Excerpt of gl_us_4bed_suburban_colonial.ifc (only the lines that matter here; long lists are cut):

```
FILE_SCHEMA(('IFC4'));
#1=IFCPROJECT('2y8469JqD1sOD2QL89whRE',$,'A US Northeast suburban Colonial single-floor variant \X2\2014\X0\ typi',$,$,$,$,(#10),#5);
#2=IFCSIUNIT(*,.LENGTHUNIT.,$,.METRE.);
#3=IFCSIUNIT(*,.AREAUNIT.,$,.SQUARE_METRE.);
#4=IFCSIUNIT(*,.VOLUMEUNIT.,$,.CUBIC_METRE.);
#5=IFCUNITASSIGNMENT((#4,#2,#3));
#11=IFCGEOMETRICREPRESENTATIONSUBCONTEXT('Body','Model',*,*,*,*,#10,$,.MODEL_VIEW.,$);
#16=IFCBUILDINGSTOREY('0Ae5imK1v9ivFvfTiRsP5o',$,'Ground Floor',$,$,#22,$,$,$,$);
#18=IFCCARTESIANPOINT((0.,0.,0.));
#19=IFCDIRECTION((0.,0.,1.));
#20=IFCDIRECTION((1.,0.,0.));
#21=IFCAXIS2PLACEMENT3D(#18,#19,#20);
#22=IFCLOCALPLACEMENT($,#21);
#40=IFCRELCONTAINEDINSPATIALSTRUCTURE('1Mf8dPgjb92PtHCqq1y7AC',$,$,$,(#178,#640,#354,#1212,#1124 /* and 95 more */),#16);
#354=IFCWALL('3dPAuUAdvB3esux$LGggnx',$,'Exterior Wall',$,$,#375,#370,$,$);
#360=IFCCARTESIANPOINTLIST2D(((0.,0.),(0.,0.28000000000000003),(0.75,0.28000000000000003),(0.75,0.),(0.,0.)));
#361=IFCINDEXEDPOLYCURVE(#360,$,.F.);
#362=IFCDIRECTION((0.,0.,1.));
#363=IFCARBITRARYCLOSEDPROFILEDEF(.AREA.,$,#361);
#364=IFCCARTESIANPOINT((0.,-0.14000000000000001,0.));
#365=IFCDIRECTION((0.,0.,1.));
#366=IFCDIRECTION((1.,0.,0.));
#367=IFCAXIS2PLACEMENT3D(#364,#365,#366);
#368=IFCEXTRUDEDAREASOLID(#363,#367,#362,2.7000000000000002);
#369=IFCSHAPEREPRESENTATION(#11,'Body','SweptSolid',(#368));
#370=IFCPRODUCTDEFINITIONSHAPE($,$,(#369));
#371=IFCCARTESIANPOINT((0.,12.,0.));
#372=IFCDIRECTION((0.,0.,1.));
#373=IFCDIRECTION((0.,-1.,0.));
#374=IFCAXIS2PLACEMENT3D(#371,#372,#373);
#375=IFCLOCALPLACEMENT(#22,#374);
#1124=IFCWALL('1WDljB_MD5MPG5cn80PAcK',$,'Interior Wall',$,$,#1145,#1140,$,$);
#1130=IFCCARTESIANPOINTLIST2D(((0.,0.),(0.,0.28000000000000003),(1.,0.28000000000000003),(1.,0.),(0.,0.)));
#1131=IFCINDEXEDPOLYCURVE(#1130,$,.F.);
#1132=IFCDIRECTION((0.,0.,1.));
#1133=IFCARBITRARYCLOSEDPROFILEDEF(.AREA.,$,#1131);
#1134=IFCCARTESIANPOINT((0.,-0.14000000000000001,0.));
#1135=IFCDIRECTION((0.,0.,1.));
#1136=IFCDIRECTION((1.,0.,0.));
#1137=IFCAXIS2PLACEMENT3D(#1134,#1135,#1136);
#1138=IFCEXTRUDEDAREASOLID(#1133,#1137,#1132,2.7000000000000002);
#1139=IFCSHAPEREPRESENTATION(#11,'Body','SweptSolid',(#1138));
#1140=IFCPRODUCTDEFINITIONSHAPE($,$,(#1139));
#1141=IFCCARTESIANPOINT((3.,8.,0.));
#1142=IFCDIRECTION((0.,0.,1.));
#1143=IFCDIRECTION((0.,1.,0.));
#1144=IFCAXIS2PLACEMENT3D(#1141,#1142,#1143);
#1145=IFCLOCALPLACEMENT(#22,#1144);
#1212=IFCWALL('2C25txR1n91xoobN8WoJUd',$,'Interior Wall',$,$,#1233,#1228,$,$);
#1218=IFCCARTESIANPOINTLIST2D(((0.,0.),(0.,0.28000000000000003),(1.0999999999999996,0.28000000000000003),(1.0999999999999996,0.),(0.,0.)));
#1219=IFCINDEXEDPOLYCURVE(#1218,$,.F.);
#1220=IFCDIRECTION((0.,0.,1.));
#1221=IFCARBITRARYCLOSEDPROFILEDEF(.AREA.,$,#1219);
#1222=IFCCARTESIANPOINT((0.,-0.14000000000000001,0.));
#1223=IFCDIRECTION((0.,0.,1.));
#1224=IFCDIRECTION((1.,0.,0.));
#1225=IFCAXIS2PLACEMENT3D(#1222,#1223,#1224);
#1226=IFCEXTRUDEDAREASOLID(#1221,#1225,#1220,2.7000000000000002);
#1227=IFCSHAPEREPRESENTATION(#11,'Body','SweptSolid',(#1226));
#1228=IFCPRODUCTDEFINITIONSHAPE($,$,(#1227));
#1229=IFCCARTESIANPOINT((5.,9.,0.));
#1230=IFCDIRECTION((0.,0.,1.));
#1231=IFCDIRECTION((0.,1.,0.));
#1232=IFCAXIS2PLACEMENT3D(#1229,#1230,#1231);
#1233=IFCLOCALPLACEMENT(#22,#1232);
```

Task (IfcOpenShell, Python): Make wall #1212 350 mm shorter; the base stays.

```python
import ifcopenshell
import ifcopenshell.geom
import ifcopenshell.util.representation
import ifcopenshell.util.shape

model = ifcopenshell.open("gl_us_4bed_suburban_colonial.ifc")
settings = ifcopenshell.geom.settings()


def volume(element):
    """Net volume in cubic metres, openings subtracted."""
    shape = ifcopenshell.geom.create_shape(settings, element)
    return ifcopenshell.util.shape.get_volume(shape.geometry)


wall = model.by_guid("2C25txR1n91xoobN8WoJUd")
before = volume(wall)

body = ifcopenshell.util.representation.get_representation(wall, "Model", "Body")
solid = body.Items[0]
old_height = solid.Depth
solid.Depth -= 0.35
after = volume(wall)

print(f"height {old_height:g} -> {solid.Depth:g}, volume {before:.3f} -> {after:.3f} m3")

model.write("gl_us_4bed_suburban_colonial_rev.ifc")
```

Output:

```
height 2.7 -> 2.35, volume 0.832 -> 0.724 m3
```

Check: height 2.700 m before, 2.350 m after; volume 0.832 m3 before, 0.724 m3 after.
